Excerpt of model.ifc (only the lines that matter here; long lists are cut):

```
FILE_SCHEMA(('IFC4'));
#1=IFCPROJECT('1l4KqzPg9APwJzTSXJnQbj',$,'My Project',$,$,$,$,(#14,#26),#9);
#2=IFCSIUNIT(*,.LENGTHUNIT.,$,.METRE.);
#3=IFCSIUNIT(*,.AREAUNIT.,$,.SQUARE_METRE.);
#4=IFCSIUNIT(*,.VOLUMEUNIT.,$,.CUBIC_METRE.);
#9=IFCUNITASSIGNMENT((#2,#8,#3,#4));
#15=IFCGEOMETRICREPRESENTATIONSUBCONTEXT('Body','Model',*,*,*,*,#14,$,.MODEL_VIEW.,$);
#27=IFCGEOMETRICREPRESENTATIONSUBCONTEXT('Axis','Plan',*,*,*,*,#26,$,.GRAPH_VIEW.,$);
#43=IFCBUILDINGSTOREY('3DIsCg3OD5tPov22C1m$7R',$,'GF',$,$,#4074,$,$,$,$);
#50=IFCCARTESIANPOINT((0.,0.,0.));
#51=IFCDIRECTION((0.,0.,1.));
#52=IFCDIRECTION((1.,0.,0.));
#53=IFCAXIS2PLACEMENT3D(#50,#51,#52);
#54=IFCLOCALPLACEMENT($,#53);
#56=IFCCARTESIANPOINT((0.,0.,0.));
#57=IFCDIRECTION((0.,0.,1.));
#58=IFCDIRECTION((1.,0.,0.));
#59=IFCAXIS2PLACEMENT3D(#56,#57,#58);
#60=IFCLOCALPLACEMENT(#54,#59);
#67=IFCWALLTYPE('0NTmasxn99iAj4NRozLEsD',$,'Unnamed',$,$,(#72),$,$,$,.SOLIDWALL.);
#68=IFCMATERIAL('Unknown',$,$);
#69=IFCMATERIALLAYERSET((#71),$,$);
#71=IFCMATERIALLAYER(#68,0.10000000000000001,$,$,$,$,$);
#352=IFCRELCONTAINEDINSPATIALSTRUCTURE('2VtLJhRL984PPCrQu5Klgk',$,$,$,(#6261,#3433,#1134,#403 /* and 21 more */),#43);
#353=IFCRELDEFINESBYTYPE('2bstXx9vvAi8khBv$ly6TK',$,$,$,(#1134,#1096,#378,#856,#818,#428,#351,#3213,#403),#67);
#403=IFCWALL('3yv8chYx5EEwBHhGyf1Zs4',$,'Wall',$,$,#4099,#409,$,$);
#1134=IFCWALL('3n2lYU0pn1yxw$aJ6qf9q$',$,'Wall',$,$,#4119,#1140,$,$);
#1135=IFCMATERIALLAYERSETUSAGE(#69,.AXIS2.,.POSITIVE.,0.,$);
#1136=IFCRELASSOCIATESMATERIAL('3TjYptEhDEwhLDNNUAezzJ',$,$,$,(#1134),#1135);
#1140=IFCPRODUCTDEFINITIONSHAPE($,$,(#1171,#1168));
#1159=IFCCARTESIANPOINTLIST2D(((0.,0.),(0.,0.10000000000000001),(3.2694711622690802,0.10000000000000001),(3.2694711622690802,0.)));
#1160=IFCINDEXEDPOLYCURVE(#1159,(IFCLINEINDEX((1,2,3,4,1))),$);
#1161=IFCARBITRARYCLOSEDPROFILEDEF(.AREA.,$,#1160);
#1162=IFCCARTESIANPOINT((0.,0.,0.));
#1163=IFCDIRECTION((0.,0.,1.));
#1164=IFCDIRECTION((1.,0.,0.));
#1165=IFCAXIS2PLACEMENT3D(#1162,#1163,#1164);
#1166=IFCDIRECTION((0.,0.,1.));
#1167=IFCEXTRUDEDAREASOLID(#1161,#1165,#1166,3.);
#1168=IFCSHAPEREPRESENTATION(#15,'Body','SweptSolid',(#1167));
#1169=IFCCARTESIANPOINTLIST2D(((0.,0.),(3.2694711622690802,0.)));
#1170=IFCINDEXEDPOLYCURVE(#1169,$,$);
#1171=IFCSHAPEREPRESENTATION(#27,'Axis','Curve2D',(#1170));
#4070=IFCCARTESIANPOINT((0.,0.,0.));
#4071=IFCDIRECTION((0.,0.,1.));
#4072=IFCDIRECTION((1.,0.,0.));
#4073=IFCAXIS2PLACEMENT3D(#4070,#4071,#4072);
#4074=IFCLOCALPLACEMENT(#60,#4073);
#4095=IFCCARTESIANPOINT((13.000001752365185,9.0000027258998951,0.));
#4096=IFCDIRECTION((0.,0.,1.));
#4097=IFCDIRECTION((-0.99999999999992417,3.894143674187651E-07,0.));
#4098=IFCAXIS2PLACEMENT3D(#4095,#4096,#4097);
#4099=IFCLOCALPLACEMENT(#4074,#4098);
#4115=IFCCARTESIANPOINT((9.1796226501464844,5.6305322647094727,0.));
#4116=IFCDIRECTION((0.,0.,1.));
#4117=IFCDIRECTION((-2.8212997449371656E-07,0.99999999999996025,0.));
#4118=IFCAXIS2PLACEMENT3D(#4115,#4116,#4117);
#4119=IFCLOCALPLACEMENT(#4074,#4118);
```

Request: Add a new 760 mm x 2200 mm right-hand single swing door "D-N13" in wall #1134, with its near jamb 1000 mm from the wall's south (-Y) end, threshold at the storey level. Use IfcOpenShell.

```python
import numpy as np
import ifcopenshell
import ifcopenshell.api.feature
import ifcopenshell.api.geometry
import ifcopenshell.api.root
import ifcopenshell.api.spatial
import ifcopenshell.geom
import ifcopenshell.util.element
import ifcopenshell.util.placement
import ifcopenshell.util.representation
import ifcopenshell.util.shape
import ifcopenshell.util.unit

model = ifcopenshell.open("model.ifc")
unit_scale = ifcopenshell.util.unit.calculate_unit_scale(model)
settings = ifcopenshell.geom.settings()


def volume(element):
    """Net volume in cubic metres, openings subtracted."""
    shape = ifcopenshell.geom.create_shape(settings, element)
    return ifcopenshell.util.shape.get_volume(shape.geometry)


wall = model.by_id(1134)
storey = ifcopenshell.util.element.get_container(wall, ifc_class="IfcBuildingStorey")
context = ifcopenshell.util.representation.get_context(model, "Model", "Body", "MODEL_VIEW")
before = volume(wall)

width, height, from_end, sill = 0.76, 2.2, 1, 0.0  # metres

# The wall runs along its own X axis, and the end named is its -X end.
wall_shape = ifcopenshell.geom.create_shape(settings, wall)
x, y, z = ifcopenshell.util.shape.get_vertices(wall_shape.geometry).T
start = x.min() + from_end
face, thickness = float(y.min()), float(y.max() - y.min())
wall_matrix = ifcopenshell.util.placement.get_local_placement(wall.ObjectPlacement)
level = ifcopenshell.util.placement.get_local_placement(storey.ObjectPlacement)[2, 3]


def in_wall(x, y):
    """Placement at x, y metres in the wall's axes, at sill height."""
    matrix = wall_matrix.copy()
    matrix[:, 3] = wall_matrix @ np.array([x / unit_scale, y / unit_scale, 0.0, 1.0])
    matrix[2, 3] = level + sill / unit_scale
    return matrix


# Opening: a box that overshoots both wall faces by 50 mm.
opening = ifcopenshell.api.root.create_entity(model, ifc_class="IfcOpeningElement", predefined_type="OPENING")
box = ifcopenshell.api.geometry.add_wall_representation(
    model, context=context, length=width, height=height, thickness=thickness + 0.1
)
ifcopenshell.api.geometry.assign_representation(model, product=opening, representation=box)
ifcopenshell.api.geometry.edit_object_placement(model, product=opening, matrix=in_wall(start, face - 0.05), is_si=False)
ifcopenshell.api.feature.add_feature(model, feature=opening, element=wall)

door = ifcopenshell.api.root.create_entity(model, ifc_class="IfcDoor", name="D-N13", predefined_type="DOOR")
door.OverallWidth, door.OverallHeight = width / unit_scale, height / unit_scale
door.OperationType = "SINGLE_SWING_RIGHT"
body = ifcopenshell.api.geometry.add_door_representation(
    model,
    context=context,
    overall_width=door.OverallWidth,
    overall_height=door.OverallHeight,
    operation_type="SINGLE_SWING_RIGHT",
    lining_properties={"LiningDepth": thickness / unit_scale, "ThresholdDepth": thickness / unit_scale},
)
ifcopenshell.api.geometry.assign_representation(model, product=door, representation=body)
ifcopenshell.api.spatial.assign_container(model, products=[door], relating_structure=storey)
ifcopenshell.api.feature.add_filling(model, opening=opening, element=door)

# The lining spans the wall, so the door starts at the wall face.
ifcopenshell.api.geometry.edit_object_placement(model, product=door, matrix=in_wall(start, face), is_si=False)

after = volume(wall)

print(f"wall volume {before:.3f} -> {after:.3f} m3")

model.write("model-out.ifc")
```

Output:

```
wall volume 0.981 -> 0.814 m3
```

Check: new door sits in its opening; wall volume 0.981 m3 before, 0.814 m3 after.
